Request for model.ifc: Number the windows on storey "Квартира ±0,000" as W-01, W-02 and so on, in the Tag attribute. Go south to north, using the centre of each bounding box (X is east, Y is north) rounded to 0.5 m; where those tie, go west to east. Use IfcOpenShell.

First a look at what the model holds.

```python
import ifcopenshell
import ifcopenshell.util.element
import ifcopenshell.util.placement

model = ifcopenshell.open("model.ifc")
print(model.schema)
storey = next(s for s in model.by_type("IfcBuildingStorey") if s.Name == "Квартира ±0,000")
windows = [e for e in ifcopenshell.util.element.get_decomposition(storey) if e.is_a("IfcWindow")]
for e in sorted(windows, key=lambda e: e.id()):
    origin = ifcopenshell.util.placement.get_local_placement(e.ObjectPlacement)[:3, 3]
    print(e.id(), e.Tag, e.Name, origin.round(2) + 0.0, sep=" | ")
```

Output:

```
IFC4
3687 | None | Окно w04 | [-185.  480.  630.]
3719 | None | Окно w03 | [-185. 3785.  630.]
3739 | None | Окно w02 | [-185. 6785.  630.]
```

```python
import ifcopenshell
import ifcopenshell.geom
import ifcopenshell.util.element
import ifcopenshell.util.shape

model = ifcopenshell.open("model.ifc")
settings = ifcopenshell.geom.settings()
settings.set("use-world-coords", True)


def centre(element):
    shape = ifcopenshell.geom.create_shape(settings, element)
    return ifcopenshell.util.shape.get_bbox_centroid(shape.geometry)


storey = next(s for s in model.by_type("IfcBuildingStorey") if s.Name == "Квартира ±0,000")
windows = [e for e in ifcopenshell.util.element.get_decomposition(storey) if e.is_a("IfcWindow")]

# Insertion points can sit at a corner or the storey origin, so sort by the geometry (in metres).
centres = {e: centre(e) for e in windows}
windows.sort(key=lambda e: (round(centres[e][1] / 0.5), centres[e][0]))

for i, e in enumerate(windows, start=1):
    number = f"W-{i:02d}"
    e.Tag = number
    print(e.id(), number)

model.write("model_updated.ifc")
```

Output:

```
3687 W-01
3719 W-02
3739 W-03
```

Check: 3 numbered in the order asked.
